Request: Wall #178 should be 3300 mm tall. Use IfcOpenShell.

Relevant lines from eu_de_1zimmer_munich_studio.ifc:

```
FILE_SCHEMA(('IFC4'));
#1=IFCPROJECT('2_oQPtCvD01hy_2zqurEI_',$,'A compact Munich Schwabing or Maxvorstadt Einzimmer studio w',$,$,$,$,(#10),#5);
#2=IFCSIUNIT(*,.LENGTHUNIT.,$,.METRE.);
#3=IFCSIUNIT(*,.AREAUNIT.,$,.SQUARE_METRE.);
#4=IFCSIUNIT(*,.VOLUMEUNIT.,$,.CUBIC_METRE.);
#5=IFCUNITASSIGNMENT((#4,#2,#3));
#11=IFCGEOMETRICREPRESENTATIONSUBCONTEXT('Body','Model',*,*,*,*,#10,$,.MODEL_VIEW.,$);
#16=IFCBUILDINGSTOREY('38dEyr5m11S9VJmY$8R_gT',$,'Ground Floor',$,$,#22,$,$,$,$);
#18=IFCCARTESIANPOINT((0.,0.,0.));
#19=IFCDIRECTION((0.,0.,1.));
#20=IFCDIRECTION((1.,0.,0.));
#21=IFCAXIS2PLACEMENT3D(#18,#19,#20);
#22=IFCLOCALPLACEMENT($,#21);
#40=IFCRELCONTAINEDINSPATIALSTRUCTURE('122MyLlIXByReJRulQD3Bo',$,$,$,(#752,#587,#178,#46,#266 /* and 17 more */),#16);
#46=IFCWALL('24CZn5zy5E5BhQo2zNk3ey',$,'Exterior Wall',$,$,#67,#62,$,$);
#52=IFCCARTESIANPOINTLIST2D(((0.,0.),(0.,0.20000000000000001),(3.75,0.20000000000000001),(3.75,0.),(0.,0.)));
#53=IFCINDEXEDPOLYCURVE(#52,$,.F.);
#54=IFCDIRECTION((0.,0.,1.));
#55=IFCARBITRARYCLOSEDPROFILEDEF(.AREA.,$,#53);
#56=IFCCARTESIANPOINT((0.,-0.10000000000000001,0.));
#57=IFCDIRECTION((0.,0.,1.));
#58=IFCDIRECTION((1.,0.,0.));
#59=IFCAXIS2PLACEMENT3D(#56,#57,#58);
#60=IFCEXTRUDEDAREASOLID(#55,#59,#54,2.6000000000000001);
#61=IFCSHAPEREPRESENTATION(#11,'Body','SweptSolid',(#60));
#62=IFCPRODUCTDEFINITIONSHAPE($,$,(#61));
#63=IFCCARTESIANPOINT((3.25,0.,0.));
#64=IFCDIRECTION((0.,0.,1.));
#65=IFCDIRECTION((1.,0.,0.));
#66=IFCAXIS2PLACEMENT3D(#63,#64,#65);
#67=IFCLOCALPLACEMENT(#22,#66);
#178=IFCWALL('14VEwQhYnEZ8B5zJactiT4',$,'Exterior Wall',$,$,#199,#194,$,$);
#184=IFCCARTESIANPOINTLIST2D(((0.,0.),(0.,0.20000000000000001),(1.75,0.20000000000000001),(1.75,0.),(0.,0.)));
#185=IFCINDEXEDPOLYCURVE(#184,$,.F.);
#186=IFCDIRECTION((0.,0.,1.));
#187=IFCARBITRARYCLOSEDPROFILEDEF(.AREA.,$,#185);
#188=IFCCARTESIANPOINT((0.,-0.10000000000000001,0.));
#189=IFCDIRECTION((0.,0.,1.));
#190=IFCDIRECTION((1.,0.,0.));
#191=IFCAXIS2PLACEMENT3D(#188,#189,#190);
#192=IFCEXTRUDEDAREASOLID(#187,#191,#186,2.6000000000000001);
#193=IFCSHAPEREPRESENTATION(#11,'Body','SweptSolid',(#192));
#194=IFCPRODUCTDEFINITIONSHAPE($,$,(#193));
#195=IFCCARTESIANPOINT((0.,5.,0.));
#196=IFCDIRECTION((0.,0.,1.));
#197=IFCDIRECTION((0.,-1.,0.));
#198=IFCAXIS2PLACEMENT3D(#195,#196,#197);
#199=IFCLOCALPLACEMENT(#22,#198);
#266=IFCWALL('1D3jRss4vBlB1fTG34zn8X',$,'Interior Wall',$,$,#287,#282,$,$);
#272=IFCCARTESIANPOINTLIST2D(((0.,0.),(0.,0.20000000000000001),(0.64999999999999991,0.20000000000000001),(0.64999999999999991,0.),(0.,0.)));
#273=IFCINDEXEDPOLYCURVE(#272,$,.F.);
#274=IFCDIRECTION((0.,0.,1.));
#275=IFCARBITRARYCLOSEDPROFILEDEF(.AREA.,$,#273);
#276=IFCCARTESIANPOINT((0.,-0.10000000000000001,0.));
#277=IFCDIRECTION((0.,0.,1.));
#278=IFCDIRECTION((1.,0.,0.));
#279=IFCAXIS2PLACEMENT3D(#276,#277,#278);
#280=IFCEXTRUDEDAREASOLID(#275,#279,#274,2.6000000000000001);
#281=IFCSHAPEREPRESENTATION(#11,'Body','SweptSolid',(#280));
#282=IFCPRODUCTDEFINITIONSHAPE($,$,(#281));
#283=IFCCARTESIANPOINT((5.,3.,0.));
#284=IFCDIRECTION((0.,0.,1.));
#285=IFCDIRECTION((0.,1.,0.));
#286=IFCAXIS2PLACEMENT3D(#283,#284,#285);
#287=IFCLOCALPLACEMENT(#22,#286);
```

```python
import ifcopenshell
import ifcopenshell.geom
import ifcopenshell.util.representation
import ifcopenshell.util.shape
import ifcopenshell.util.unit

model = ifcopenshell.open("eu_de_1zimmer_munich_studio.ifc")
unit_scale = ifcopenshell.util.unit.calculate_unit_scale(model)
settings = ifcopenshell.geom.settings()


def volume(element):
    """Net volume in cubic metres, openings subtracted."""
    shape = ifcopenshell.geom.create_shape(settings, element)
    return ifcopenshell.util.shape.get_volume(shape.geometry)


wall = model.by_id(178)
before = volume(wall)

body = ifcopenshell.util.representation.get_representation(wall, "Model", "Body")
solid = body.Items[0]
old_height = solid.Depth
solid.Depth = 3.3 / unit_scale
after = volume(wall)

print(f"height {old_height:g} -> {solid.Depth:g}, volume {before:.3f} -> {after:.3f} m3")

model.write("eu_de_1zimmer_munich_studio_rev.ifc")
```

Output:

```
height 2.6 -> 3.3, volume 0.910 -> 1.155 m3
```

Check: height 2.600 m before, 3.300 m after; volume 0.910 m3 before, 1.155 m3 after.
